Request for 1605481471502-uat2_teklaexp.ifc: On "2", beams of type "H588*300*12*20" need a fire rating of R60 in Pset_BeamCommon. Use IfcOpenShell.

First a look at what the model holds.

```python
import ifcopenshell
import ifcopenshell.util.element

model = ifcopenshell.open("1605481471502-uat2_teklaexp.ifc")
print(model.schema)
storey = next(s for s in model.by_type("IfcBuildingStorey") if s.Name == "2")
beams = [e for e in ifcopenshell.util.element.get_decomposition(storey) if e.is_a("IfcBeam")]
seen = {}
for e in beams:
    element_type = ifcopenshell.util.element.get_type(e)
    key = (element_type.Name if element_type != e and element_type else None, ifcopenshell.util.element.get_pset(e, "Pset_BeamCommon", "FireRating"))
    seen[key] = seen.get(key, 0) + 1
for (name, value), count in sorted(seen.items(), key=str):
    print(count, "x", name, "|", value)
```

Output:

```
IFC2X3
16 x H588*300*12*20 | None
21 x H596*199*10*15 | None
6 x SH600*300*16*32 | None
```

```python
import ifcopenshell
import ifcopenshell.api.pset
import ifcopenshell.util.element

model = ifcopenshell.open("1605481471502-uat2_teklaexp.ifc")

storey = next(s for s in model.by_type("IfcBuildingStorey") if s.Name == "2")
beams = [e for e in ifcopenshell.util.element.get_decomposition(storey) if e.is_a("IfcBeam")]

count = 0
for e in beams:
    element_type = ifcopenshell.util.element.get_type(e)
    if element_type in (None, e) or element_type.Name != "H588*300*12*20":
        continue
    found = ifcopenshell.util.element.get_pset(e, "Pset_BeamCommon", should_inherit=False)
    if found:
        pset = model.by_id(found["id"])
        if len(ifcopenshell.util.element.get_elements_by_pset(pset)) > 1:
            pset = ifcopenshell.api.pset.unshare_pset(model, products=[e], pset=pset)[0]
    else:
        pset = ifcopenshell.api.pset.add_pset(model, product=e, name="Pset_BeamCommon")
    ifcopenshell.api.pset.edit_pset(model, pset=pset, properties={"FireRating": "R60"})
    count += 1

print(count, "beams updated")

model.write("1605481471502-uat2_teklaexp_updated.ifc")
```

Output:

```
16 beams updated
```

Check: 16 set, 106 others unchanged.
